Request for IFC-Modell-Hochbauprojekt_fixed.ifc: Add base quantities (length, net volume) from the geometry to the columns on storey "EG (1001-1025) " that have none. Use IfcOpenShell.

First a look at what the model holds.

```python
import ifcopenshell
import ifcopenshell.util.element
import ifcopenshell.util.unit

model = ifcopenshell.open("IFC-Modell-Hochbauprojekt_fixed.ifc")
print(model.schema)
for unit_type in ("LENGTHUNIT", "AREAUNIT", "VOLUMEUNIT"):
    print(unit_type, ifcopenshell.util.unit.calculate_unit_scale(model, unit_type))
storey = next(s for s in model.by_type("IfcBuildingStorey") if s.Name == "EG (1001-1025) ")
columns = [e for e in ifcopenshell.util.element.get_decomposition(storey) if e.is_a("IfcColumn")]
for e in sorted(columns, key=lambda e: e.id()):
    print(e.id(), e.is_a(), e.Name, list(ifcopenshell.util.element.get_psets(e, qtos_only=True)), sep=" | ")
```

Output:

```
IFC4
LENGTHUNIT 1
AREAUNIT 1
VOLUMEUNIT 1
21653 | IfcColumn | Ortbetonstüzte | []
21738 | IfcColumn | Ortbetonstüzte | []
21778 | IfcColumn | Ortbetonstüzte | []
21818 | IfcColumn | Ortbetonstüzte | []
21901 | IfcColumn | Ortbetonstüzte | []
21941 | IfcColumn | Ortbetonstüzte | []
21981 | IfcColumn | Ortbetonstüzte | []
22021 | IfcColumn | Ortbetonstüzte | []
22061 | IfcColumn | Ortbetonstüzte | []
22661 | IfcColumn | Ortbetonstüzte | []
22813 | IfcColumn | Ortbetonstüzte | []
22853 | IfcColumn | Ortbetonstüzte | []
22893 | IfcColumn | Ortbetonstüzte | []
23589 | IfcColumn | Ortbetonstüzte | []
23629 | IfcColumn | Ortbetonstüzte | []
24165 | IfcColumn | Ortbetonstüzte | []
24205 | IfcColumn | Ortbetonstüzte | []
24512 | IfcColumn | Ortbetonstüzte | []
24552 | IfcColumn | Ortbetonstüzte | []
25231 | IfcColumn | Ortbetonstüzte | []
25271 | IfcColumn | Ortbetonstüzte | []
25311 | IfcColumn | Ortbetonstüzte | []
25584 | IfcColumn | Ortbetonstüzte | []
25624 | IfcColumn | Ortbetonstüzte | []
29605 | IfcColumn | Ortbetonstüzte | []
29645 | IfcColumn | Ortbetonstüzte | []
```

```python
import ifcopenshell
import ifcopenshell.api.pset
import ifcopenshell.geom
import ifcopenshell.util.element
import ifcopenshell.util.shape
import ifcopenshell.util.unit

model = ifcopenshell.open("IFC-Modell-Hochbauprojekt_fixed.ifc")
unit_scale = ifcopenshell.util.unit.calculate_unit_scale(model)
volume_scale = ifcopenshell.util.unit.calculate_unit_scale(model, "VOLUMEUNIT")
settings = ifcopenshell.geom.settings()

storey = next(s for s in model.by_type("IfcBuildingStorey") if s.Name == "EG (1001-1025) ")
columns = [e for e in ifcopenshell.util.element.get_decomposition(storey) if e.is_a("IfcColumn")]

for e in sorted(columns, key=lambda e: e.id()):
    if ifcopenshell.util.element.get_psets(e, qtos_only=True, should_inherit=False):
        continue
    # Geometry comes back in metres, in the element's own axes.
    shape = ifcopenshell.geom.create_shape(settings, e)
    values = {
        "Length": ifcopenshell.util.shape.get_z(shape.geometry) / unit_scale,
        "NetVolume": ifcopenshell.util.shape.get_volume(shape.geometry) / volume_scale,
    }
    qto = ifcopenshell.api.pset.add_qto(model, product=e, name="Qto_ColumnBaseQuantities")
    ifcopenshell.api.pset.edit_qto(model, qto=qto, properties=values)
    print(e.id(), {k: round(v, 3) for k, v in values.items()})

model.write("IFC-Modell-Hochbauprojekt_fixed_edited.ifc")
```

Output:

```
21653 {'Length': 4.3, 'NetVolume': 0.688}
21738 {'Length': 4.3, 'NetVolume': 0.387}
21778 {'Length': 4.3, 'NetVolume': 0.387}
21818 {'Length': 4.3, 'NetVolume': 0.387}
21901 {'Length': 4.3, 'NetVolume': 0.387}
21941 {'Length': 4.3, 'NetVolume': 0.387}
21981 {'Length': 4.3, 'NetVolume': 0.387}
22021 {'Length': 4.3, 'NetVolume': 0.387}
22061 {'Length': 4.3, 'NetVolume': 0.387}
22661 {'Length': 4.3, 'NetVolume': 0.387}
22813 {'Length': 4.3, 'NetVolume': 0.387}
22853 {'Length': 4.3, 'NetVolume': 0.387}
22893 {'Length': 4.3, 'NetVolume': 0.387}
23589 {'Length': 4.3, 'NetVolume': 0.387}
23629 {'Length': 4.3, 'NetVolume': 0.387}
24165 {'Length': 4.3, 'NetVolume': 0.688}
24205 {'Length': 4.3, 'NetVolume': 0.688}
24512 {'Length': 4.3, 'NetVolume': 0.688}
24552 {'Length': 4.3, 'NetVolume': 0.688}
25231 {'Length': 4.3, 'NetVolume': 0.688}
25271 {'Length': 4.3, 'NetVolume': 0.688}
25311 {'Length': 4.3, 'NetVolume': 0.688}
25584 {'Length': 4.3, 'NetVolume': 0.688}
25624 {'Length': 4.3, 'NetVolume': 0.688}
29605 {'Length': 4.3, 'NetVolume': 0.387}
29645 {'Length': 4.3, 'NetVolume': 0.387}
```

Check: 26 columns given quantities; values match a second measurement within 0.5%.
